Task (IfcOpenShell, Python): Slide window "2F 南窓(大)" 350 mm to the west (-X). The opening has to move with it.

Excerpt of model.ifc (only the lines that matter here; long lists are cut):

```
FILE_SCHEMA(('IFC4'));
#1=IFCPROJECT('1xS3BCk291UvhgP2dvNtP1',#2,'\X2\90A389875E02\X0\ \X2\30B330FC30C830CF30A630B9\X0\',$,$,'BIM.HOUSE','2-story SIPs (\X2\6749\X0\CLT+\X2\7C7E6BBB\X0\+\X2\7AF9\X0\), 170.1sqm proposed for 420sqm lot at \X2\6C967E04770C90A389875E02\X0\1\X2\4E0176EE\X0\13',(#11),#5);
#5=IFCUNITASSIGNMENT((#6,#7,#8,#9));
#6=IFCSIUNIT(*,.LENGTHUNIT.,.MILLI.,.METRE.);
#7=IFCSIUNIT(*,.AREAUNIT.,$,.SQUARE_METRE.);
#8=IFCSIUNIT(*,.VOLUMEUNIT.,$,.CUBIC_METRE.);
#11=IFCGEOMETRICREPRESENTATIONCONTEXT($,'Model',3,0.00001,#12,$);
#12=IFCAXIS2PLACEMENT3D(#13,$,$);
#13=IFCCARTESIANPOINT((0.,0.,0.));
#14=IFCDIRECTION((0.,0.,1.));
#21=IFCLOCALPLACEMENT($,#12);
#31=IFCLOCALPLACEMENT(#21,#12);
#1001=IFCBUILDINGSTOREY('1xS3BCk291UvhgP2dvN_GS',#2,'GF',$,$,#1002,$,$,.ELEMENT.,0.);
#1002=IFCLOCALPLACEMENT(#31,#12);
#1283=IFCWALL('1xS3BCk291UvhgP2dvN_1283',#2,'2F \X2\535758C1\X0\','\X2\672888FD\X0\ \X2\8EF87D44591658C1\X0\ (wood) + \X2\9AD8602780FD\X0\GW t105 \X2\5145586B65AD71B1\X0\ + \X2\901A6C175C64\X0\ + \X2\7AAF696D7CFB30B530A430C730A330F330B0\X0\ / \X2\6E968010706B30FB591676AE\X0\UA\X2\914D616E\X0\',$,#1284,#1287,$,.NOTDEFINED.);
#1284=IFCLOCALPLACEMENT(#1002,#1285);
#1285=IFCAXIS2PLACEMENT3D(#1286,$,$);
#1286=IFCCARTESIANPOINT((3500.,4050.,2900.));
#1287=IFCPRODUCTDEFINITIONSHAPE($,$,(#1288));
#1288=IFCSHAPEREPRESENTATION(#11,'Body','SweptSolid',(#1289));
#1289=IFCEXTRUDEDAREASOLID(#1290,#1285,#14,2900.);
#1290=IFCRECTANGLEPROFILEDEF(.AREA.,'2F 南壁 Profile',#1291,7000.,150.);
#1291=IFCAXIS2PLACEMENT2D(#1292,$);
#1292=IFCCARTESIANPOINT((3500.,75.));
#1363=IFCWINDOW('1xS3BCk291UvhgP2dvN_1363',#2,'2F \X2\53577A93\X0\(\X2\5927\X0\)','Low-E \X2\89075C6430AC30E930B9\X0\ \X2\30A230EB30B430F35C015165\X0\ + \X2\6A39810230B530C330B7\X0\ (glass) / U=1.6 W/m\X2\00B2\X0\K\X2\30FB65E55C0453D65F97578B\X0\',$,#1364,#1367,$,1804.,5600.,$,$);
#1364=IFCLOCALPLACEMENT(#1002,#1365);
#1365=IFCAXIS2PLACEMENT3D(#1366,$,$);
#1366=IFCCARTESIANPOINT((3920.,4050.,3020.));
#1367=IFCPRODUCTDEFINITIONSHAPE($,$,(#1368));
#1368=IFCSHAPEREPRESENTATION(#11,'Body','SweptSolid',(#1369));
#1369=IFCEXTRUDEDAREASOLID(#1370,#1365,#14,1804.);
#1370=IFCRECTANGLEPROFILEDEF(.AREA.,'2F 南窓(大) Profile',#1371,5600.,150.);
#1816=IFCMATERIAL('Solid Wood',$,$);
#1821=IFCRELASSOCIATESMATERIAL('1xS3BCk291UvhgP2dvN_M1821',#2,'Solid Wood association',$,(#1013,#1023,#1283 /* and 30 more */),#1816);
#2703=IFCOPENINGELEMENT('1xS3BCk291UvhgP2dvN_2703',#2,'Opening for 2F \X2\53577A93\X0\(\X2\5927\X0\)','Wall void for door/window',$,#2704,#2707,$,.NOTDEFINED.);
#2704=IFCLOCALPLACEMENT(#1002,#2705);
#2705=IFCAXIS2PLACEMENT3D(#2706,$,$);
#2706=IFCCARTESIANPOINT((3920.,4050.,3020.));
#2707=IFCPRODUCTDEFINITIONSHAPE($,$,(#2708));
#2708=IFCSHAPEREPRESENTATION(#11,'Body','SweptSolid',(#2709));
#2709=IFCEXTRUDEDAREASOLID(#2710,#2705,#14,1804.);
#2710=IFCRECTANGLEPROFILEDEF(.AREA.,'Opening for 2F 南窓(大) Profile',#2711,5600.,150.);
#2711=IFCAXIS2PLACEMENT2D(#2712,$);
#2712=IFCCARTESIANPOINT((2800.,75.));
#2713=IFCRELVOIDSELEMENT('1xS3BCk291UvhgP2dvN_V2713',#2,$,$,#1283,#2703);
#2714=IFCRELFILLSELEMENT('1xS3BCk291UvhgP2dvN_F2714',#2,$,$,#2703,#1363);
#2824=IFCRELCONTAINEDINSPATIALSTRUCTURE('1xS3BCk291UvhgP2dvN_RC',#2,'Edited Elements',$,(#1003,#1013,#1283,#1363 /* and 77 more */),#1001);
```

```python
import ifcopenshell
import ifcopenshell.api.geometry
import ifcopenshell.util.placement

model = ifcopenshell.open("model.ifc")

window = model.by_id(1363)
opening = window.FillsVoids[0].RelatingOpeningElement
wall = opening.VoidsElements[0].RelatingBuildingElement

wall_matrix = ifcopenshell.util.placement.get_local_placement(wall.ObjectPlacement)
shift = wall_matrix[:3, 0] * -350.0
before = ifcopenshell.util.placement.get_local_placement(window.ObjectPlacement)[:3, 3].copy()

# The window is not placed relative to its opening, so move both.
for product in (opening, window):
    matrix = ifcopenshell.util.placement.get_local_placement(product.ObjectPlacement)
    matrix[:3, 3] += shift
    ifcopenshell.api.geometry.edit_object_placement(model, product=product, matrix=matrix, is_si=False)

after = ifcopenshell.util.placement.get_local_placement(window.ObjectPlacement)[:3, 3]
print("window moved by", (after - before).round(3) + 0.0)

model.write("model_v2.ifc")
```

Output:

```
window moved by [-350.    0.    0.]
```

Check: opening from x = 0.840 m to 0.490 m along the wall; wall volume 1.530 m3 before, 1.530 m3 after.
